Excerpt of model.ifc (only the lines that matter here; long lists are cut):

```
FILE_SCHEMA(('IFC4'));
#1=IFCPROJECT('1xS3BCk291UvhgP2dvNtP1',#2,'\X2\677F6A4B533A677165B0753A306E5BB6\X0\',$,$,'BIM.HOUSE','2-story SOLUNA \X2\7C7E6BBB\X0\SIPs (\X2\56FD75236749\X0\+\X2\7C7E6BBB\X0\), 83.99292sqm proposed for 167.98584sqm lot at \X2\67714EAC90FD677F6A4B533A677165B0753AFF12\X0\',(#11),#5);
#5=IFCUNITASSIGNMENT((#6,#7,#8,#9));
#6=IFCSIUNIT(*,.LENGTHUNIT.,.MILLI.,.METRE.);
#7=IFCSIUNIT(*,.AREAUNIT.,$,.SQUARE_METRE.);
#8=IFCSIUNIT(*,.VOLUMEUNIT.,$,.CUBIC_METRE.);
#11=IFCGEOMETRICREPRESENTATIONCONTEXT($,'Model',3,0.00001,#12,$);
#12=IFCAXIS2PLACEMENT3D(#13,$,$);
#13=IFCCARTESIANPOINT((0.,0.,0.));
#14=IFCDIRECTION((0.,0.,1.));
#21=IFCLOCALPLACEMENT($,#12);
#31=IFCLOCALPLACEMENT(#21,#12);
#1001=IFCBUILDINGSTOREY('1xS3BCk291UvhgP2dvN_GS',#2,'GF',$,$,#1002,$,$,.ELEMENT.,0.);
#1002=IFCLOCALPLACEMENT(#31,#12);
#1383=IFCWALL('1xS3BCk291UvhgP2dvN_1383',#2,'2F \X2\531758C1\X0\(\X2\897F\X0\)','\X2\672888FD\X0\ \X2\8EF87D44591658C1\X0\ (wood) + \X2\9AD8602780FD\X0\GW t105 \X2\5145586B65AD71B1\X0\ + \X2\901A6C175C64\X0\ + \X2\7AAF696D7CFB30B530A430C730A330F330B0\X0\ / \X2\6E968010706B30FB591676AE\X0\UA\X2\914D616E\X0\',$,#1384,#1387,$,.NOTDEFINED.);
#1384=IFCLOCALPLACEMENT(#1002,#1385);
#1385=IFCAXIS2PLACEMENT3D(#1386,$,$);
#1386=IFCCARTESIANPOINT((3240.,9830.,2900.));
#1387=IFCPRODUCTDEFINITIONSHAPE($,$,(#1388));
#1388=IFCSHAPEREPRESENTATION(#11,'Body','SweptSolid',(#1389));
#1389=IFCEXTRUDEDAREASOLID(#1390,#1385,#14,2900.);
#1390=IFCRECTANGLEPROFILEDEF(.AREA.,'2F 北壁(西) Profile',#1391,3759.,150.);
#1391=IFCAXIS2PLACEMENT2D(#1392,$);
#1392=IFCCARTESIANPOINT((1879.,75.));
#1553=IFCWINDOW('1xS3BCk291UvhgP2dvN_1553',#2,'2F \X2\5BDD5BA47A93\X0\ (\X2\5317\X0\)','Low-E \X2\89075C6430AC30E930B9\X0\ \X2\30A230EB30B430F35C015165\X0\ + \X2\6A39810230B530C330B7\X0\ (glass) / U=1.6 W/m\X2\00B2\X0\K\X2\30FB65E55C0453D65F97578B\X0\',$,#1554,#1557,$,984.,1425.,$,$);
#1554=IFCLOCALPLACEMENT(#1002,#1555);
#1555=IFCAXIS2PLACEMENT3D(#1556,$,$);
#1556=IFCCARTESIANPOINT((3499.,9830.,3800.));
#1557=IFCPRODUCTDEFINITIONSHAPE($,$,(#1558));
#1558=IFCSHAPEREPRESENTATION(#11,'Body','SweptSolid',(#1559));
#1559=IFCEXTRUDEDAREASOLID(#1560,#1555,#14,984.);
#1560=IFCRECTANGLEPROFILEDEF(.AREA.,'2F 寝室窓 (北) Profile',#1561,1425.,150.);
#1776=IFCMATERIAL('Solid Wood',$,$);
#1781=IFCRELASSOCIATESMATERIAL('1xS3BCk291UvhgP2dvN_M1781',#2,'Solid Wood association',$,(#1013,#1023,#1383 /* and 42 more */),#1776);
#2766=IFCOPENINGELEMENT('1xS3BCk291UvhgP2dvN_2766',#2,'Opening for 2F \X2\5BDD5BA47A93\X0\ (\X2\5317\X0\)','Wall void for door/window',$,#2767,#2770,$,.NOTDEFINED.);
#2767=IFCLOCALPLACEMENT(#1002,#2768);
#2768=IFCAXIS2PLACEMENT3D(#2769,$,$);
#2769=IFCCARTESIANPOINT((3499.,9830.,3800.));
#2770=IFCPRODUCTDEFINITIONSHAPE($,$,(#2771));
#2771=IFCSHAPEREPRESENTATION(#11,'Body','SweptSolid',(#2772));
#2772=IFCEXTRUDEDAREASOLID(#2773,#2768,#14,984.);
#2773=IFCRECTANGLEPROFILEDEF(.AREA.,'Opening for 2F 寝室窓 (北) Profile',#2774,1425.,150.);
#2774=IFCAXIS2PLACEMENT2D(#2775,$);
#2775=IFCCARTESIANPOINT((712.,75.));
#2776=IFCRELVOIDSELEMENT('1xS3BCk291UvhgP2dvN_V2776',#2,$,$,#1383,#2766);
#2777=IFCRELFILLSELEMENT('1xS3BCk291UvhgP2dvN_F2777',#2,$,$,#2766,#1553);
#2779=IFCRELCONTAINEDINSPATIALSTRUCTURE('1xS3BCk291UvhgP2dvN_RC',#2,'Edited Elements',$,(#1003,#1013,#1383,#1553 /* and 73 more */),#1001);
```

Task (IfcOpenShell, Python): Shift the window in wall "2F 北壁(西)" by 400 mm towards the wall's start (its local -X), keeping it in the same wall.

```python
import ifcopenshell
import ifcopenshell.api.geometry
import ifcopenshell.util.placement
import ifcopenshell.util.unit

model = ifcopenshell.open("model.ifc")
unit_scale = ifcopenshell.util.unit.calculate_unit_scale(model)

window = model.by_guid("1xS3BCk291UvhgP2dvN_1553")
opening = window.FillsVoids[0].RelatingOpeningElement
wall = opening.VoidsElements[0].RelatingBuildingElement

wall_matrix = ifcopenshell.util.placement.get_local_placement(wall.ObjectPlacement)
shift = wall_matrix[:3, 0] * -0.4 / unit_scale
before = ifcopenshell.util.placement.get_local_placement(window.ObjectPlacement)[:3, 3].copy()

# The window is not placed relative to its opening, so move both.
for product in (opening, window):
    matrix = ifcopenshell.util.placement.get_local_placement(product.ObjectPlacement)
    matrix[:3, 3] += shift
    ifcopenshell.api.geometry.edit_object_placement(model, product=product, matrix=matrix, is_si=False)

after = ifcopenshell.util.placement.get_local_placement(window.ObjectPlacement)[:3, 3]
print("window moved by", (after - before).round(3) + 0.0)

model.write("model-out.ifc")
```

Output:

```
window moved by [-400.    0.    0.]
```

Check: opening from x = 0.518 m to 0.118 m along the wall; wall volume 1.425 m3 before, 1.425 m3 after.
